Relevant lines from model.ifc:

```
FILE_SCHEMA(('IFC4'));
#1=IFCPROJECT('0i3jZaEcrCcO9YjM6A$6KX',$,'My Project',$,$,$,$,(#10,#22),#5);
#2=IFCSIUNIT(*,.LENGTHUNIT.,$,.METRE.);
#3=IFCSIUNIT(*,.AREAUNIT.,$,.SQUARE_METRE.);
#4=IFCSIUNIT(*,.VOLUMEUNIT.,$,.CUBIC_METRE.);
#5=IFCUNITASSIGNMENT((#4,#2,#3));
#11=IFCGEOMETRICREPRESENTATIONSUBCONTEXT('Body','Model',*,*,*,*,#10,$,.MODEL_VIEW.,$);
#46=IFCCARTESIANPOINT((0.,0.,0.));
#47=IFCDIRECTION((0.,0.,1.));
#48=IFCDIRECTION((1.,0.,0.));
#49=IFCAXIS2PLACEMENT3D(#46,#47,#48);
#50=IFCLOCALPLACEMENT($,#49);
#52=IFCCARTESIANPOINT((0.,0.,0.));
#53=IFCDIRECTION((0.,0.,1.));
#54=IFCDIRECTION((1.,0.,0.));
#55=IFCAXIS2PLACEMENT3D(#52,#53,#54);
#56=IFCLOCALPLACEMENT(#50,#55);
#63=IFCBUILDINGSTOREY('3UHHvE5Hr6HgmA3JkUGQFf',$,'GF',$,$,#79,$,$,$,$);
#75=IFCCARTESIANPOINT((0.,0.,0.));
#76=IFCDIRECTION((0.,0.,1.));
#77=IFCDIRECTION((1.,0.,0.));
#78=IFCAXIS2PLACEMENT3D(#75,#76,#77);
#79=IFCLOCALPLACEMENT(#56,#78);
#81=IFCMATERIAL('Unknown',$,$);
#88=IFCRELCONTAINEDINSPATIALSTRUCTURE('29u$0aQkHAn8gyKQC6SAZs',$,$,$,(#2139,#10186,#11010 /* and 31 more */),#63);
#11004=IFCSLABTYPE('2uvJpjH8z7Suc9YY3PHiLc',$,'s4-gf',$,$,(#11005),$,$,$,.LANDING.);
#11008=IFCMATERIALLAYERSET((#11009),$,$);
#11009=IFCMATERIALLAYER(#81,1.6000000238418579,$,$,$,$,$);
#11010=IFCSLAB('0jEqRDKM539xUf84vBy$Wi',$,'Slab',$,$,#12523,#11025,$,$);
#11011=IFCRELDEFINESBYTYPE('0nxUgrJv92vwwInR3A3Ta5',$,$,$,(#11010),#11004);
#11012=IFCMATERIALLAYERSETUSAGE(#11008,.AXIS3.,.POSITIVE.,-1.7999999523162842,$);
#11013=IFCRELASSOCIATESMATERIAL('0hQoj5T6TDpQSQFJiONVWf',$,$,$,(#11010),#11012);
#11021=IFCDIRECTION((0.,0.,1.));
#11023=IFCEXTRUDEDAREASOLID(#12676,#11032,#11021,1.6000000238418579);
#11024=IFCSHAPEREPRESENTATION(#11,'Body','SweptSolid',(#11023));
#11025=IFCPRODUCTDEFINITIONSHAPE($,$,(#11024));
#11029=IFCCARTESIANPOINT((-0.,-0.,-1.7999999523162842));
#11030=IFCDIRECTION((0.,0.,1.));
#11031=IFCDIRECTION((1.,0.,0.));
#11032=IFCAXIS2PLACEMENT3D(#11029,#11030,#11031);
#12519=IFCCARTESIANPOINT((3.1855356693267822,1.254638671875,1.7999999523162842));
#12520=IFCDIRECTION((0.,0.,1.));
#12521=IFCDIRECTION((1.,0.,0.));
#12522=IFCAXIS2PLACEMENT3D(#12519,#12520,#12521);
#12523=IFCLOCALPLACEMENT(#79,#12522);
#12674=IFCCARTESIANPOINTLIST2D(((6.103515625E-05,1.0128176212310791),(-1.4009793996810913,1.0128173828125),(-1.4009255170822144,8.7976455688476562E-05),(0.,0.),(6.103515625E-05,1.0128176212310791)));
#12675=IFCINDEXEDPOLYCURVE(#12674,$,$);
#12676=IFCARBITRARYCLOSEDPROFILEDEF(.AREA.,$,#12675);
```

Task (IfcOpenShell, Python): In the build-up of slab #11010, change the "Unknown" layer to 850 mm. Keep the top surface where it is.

```python
import ifcopenshell
import ifcopenshell.util.element
import ifcopenshell.util.representation

model = ifcopenshell.open("model.ifc")

layer_set = model.by_id(11008)
layer = next(l for l in layer_set.MaterialLayers if l.Material and l.Material.Name == "Unknown")
change = 0.85 - layer.LayerThickness
layer.LayerThickness += change

# Geometry does not follow the layer set by itself.
slabs = [e for e in ifcopenshell.util.element.get_elements_by_material(model, layer_set) if e.is_a("IfcSlab")]
for slab in sorted(slabs, key=lambda e: e.id()):
    body = ifcopenshell.util.representation.get_representation(slab, "Model", "Body")
    solid = body.Items[0]
    old_depth = solid.Depth
    solid.Depth += change
    # Extruded upwards: lower the start of the extrusion so the top stays.
    x, y, z = solid.Position.Location.Coordinates
    solid.Position.Location = model.createIfcCartesianPoint((x, y, z - change))
    print(slab.id(), f"{old_depth:g} -> {solid.Depth:g}")

# The layers are counted up from the underside, which has moved.
for usage in {ifcopenshell.util.element.get_material(slab) for slab in slabs}:
    usage.OffsetFromReferenceLine -= change

model.write("model_v2.ifc")
```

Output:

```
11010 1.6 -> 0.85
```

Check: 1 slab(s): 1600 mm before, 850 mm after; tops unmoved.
